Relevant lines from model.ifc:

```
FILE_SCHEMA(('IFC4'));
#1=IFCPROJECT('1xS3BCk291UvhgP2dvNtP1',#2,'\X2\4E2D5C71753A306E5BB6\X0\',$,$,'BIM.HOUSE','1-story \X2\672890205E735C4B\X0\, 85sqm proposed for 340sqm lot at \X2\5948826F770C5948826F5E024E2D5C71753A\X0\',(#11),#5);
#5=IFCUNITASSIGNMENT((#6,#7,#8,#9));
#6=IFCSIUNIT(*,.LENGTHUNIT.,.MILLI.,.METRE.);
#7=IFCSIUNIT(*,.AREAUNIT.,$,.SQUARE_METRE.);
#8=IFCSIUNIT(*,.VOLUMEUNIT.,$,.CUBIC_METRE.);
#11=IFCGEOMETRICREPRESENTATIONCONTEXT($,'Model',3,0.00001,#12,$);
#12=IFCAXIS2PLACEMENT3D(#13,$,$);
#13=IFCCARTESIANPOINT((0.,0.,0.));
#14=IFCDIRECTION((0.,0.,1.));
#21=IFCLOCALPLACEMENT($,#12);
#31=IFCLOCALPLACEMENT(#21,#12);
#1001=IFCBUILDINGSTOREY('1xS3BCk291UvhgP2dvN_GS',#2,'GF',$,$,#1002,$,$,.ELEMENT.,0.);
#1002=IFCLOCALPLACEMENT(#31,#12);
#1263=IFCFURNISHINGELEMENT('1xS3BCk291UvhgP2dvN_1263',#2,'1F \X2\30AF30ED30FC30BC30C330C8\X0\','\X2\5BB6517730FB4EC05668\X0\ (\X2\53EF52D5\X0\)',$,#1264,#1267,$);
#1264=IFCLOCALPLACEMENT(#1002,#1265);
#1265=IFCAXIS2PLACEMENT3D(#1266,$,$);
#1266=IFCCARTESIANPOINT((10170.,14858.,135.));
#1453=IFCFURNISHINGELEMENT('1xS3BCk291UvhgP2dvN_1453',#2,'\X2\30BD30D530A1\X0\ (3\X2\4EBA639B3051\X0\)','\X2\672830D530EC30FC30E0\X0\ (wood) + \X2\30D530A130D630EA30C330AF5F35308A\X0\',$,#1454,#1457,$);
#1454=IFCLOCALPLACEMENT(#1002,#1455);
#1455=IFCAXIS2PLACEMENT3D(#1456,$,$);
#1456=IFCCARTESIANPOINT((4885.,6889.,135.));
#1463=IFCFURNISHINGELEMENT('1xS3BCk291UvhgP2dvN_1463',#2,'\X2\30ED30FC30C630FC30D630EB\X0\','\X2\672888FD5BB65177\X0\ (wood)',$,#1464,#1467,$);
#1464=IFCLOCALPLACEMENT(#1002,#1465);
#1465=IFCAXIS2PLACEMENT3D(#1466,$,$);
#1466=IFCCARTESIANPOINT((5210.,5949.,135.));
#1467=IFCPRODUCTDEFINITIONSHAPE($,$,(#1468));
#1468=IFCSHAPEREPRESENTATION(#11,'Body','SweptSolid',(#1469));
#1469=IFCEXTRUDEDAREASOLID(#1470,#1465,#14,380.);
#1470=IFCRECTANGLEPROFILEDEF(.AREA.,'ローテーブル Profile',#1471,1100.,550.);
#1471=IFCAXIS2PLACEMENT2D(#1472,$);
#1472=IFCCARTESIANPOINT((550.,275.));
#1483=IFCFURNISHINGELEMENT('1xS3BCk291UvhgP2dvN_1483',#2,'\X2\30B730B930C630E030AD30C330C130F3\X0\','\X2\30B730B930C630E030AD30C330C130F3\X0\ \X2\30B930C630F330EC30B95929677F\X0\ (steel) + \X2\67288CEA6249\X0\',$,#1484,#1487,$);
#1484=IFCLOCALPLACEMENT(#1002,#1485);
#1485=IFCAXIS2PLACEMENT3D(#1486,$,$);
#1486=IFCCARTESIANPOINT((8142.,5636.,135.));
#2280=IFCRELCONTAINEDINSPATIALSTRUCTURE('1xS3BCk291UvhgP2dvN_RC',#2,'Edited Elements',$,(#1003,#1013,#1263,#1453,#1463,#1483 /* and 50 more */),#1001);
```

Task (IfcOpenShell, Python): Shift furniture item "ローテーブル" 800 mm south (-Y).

```python
import ifcopenshell
import ifcopenshell.api.geometry
import ifcopenshell.util.placement

model = ifcopenshell.open("model.ifc")

item = model.by_guid("1xS3BCk291UvhgP2dvN_1463")
matrix = ifcopenshell.util.placement.get_local_placement(item.ObjectPlacement)
matrix[1, 3] -= 800.0
ifcopenshell.api.geometry.edit_object_placement(model, product=item, matrix=matrix, is_si=False)

print(ifcopenshell.util.placement.get_local_placement(item.ObjectPlacement).round(3) + 0.0)

model.write("model_rev.ifc")
```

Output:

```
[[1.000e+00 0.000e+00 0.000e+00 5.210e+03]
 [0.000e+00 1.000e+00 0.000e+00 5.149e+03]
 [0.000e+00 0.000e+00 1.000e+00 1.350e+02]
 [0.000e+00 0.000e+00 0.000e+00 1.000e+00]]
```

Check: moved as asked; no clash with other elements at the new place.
